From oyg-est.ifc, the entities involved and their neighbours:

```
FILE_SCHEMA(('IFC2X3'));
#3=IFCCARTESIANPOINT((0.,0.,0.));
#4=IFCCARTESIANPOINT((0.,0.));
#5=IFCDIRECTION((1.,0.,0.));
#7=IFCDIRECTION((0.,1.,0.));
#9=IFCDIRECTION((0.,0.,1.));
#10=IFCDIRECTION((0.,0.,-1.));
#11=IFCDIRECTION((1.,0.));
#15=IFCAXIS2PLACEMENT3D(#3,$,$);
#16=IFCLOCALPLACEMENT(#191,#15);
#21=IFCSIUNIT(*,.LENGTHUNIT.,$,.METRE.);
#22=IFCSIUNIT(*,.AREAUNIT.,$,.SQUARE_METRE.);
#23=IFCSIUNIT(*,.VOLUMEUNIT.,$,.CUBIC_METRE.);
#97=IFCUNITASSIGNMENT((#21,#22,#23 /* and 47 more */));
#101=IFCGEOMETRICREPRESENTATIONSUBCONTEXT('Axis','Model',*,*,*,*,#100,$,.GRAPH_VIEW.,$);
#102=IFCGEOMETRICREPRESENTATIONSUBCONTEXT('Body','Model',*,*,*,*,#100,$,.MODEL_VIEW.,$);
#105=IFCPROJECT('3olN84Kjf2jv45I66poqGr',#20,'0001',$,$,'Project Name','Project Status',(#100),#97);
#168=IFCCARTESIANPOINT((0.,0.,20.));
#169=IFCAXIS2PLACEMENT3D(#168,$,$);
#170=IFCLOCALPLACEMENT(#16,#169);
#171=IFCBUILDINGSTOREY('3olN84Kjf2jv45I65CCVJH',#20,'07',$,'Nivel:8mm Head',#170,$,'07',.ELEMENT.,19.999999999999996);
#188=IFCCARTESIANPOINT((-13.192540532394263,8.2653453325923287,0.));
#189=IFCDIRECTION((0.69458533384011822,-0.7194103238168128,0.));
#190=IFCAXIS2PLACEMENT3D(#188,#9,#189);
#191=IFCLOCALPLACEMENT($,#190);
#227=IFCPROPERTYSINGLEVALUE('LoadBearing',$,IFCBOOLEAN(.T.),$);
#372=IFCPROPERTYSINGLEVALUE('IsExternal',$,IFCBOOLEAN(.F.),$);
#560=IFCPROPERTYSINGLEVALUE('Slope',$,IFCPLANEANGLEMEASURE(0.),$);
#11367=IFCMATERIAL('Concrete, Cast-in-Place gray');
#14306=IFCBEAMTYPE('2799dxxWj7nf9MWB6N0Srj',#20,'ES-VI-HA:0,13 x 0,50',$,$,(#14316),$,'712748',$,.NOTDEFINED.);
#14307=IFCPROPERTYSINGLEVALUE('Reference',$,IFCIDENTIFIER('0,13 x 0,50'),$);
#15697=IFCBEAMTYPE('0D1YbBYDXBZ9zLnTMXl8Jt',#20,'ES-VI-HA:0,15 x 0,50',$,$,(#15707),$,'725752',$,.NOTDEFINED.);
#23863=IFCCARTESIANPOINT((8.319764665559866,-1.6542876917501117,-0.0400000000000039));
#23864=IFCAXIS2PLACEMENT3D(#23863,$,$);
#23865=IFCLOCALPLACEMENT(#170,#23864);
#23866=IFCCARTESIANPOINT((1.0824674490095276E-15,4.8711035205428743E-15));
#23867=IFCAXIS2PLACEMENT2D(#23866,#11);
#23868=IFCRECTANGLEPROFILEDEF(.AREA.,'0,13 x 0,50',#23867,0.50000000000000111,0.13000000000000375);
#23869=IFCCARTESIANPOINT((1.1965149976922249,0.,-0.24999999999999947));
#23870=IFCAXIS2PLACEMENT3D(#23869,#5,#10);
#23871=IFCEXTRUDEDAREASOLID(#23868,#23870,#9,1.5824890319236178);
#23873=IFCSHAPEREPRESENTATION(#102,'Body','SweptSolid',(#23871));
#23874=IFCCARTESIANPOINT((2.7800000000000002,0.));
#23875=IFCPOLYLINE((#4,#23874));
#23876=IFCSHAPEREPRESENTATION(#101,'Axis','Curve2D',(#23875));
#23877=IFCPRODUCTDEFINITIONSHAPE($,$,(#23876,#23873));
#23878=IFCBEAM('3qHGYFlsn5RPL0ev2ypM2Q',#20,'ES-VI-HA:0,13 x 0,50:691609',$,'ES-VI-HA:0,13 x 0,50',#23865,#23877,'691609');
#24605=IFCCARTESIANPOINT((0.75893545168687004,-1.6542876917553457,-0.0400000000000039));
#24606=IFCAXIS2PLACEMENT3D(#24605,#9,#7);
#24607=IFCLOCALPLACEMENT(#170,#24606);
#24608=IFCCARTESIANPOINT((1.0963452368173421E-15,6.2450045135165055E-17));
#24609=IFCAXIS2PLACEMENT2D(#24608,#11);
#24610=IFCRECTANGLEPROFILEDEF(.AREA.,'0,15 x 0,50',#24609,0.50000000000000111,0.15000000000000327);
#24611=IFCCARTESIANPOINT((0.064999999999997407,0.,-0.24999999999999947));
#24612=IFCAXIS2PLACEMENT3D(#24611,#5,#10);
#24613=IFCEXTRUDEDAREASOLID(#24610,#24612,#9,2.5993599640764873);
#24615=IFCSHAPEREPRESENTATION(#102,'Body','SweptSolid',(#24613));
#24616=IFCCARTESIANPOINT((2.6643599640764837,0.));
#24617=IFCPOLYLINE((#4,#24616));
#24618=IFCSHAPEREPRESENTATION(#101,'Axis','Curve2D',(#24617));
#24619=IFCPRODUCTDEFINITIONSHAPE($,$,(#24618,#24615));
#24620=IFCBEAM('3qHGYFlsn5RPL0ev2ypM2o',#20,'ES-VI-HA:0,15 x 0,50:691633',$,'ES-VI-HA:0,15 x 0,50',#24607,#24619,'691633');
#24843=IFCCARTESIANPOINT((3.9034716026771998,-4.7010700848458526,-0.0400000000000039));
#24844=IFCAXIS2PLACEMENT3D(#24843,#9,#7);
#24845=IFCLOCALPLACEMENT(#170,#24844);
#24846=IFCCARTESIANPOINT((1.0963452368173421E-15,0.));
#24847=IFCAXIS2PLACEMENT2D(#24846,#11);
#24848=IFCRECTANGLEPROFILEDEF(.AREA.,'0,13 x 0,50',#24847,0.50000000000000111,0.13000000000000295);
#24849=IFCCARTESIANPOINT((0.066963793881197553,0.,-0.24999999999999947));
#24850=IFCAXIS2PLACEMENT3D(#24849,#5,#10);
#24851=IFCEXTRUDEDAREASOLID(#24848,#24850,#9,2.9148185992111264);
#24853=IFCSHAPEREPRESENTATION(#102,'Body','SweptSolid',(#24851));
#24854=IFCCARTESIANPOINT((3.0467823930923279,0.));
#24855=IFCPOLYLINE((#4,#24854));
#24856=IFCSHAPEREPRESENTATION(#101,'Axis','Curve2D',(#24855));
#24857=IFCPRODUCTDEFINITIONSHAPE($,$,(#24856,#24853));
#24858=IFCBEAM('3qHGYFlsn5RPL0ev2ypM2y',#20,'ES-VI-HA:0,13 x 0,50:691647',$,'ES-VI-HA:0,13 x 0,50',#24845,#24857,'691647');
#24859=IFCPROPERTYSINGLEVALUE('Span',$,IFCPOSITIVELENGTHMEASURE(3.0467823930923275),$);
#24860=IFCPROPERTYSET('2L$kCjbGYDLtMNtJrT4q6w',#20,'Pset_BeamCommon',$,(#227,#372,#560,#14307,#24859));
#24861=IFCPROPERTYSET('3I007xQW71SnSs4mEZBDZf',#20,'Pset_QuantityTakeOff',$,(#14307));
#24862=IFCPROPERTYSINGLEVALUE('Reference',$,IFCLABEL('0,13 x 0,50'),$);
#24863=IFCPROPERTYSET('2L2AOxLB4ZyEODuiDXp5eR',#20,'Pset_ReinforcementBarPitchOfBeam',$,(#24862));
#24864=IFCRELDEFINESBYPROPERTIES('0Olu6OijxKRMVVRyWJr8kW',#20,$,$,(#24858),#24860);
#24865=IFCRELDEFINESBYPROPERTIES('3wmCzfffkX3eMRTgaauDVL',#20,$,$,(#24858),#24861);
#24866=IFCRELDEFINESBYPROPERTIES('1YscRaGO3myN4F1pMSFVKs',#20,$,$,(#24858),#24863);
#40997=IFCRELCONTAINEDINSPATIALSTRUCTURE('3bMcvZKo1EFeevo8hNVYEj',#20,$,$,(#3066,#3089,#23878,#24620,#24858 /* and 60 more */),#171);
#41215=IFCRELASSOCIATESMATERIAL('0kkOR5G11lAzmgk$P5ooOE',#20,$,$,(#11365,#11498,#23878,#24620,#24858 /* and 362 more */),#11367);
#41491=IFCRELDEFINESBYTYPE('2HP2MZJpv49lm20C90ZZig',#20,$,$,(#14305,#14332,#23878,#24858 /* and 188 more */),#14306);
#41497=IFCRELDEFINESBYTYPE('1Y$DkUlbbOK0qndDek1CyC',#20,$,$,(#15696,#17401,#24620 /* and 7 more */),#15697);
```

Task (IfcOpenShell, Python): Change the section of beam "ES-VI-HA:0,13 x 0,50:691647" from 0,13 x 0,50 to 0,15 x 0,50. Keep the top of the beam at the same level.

```python
import ifcopenshell
import ifcopenshell.api.pset
import ifcopenshell.api.type
import ifcopenshell.util.element
import ifcopenshell.util.representation

model = ifcopenshell.open("oyg-est.ifc")

member = model.by_guid("3qHGYFlsn5RPL0ev2ypM2y")
source = next(p for p in model.by_type("IfcRectangleProfileDef") if p.ProfileName == "0,15 x 0,50")

body = ifcopenshell.util.representation.get_representation(member, "Model", "Body")
solid = body.Items[0]
old_profile = solid.SweptArea

# Copy the section's sizes but keep this member's own profile position.
profile = ifcopenshell.util.element.copy(model, source)
# Profiles are centred, so shift by half the change in depth to hold the top.
shift = (old_profile.XDim - profile.XDim) / 2
x, y = old_profile.Position.Location.Coordinates
up = (-1.0, 0.0)  # upwards, in the solid's own plane
location = model.createIfcCartesianPoint((x + up[0] * shift, y + up[1] * shift))
profile.Position = model.createIfcAxis2Placement2D(location, old_profile.Position.RefDirection)
solid.SweptArea = profile
if not model.get_total_inverses(old_profile):
    ifcopenshell.util.element.remove_deep2(model, old_profile)

new_type = model.by_guid("0D1YbBYDXBZ9zLnTMXl8Jt")
ifcopenshell.api.type.assign_type(
    model, related_objects=[member], relating_type=new_type, should_map_representations=False
)
member.Name = member.Name.replace("0,13 x 0,50", "0,15 x 0,50")
member.ObjectType = "ES-VI-HA:0,15 x 0,50"
pset = model.by_id(ifcopenshell.util.element.get_pset(member, "Pset_BeamCommon", should_inherit=False)["id"])
ifcopenshell.api.pset.edit_pset(model, pset=pset, properties={"Reference": "0,15 x 0,50"})
pset = model.by_id(ifcopenshell.util.element.get_pset(member, "Pset_QuantityTakeOff", should_inherit=False)["id"])
ifcopenshell.api.pset.edit_pset(model, pset=pset, properties={"Reference": "0,15 x 0,50"})
pset = model.by_id(ifcopenshell.util.element.get_pset(member, "Pset_ReinforcementBarPitchOfBeam", should_inherit=False)["id"])
ifcopenshell.api.pset.edit_pset(model, pset=pset, properties={"Reference": "0,15 x 0,50"})

print(solid.SweptArea)

model.write("oyg-est_updated.ifc")
```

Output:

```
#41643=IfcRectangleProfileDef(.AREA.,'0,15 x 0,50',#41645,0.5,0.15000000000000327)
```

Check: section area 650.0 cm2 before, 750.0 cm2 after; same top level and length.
